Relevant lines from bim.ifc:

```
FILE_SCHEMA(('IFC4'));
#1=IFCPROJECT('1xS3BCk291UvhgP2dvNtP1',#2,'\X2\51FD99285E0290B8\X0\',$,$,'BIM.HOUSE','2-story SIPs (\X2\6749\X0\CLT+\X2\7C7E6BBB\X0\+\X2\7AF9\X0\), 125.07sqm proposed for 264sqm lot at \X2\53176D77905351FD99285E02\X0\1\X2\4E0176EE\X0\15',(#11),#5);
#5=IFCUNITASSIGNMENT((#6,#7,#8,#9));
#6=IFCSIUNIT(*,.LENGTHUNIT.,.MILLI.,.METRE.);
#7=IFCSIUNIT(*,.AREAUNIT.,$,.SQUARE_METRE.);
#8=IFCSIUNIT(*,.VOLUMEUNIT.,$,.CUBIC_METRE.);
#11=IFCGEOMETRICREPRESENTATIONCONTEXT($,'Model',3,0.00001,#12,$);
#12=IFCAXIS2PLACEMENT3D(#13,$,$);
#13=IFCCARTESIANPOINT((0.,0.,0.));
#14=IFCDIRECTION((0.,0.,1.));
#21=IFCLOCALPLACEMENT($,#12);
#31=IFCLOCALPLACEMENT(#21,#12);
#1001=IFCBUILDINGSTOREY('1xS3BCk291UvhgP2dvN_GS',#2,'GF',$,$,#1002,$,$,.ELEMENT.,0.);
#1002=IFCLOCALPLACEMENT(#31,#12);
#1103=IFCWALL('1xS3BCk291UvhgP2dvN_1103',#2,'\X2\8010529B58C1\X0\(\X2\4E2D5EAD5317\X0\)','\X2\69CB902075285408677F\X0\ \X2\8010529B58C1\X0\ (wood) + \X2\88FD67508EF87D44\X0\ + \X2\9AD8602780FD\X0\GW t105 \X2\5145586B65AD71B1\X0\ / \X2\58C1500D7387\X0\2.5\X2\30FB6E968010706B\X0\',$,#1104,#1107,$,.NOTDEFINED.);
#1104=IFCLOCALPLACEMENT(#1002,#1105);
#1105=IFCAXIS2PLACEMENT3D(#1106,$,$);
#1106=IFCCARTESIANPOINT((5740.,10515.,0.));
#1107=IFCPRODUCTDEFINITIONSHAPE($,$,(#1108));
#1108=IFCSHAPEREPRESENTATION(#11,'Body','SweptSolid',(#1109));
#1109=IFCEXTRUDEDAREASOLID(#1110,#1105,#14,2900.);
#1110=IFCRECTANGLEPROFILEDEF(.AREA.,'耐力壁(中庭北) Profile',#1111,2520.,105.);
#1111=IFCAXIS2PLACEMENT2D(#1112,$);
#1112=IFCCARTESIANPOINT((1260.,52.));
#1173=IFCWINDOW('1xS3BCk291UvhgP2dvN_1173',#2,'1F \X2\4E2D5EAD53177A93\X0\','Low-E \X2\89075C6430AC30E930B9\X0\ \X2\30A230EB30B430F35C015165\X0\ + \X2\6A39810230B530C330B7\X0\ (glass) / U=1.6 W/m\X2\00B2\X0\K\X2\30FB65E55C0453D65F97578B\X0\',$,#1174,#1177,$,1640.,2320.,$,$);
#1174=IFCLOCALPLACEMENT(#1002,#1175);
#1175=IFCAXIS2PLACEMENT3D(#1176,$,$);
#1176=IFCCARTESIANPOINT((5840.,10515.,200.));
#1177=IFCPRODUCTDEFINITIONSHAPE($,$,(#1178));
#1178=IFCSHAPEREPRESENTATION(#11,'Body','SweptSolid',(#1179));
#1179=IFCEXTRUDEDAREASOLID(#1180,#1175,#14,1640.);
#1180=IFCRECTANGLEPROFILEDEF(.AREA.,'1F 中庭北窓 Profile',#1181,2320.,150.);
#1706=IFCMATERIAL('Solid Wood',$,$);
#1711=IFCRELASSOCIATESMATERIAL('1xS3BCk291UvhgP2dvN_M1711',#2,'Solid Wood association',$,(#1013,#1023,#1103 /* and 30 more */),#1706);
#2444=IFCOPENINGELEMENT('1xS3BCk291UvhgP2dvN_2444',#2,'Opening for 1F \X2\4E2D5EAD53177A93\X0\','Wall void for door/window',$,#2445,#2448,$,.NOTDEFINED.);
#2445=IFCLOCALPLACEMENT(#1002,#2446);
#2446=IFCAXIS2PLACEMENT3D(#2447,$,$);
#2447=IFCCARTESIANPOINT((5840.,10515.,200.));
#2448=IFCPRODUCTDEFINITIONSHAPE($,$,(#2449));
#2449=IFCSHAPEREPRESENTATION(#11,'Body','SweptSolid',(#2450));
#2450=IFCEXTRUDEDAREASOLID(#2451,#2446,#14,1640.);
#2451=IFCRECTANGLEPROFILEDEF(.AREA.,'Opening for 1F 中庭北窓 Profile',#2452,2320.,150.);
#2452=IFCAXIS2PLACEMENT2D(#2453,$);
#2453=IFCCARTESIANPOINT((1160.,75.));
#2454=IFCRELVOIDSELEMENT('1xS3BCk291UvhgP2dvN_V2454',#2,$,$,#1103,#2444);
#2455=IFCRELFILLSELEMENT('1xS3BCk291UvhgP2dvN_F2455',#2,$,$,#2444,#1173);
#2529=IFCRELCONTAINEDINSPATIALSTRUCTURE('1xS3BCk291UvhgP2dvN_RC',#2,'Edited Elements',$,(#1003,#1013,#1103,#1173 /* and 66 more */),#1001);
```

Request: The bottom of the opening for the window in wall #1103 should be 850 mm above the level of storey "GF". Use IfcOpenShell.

```python
import numpy as np
import ifcopenshell
import ifcopenshell.api.geometry
import ifcopenshell.geom
import ifcopenshell.util.element
import ifcopenshell.util.placement
import ifcopenshell.util.shape
import ifcopenshell.util.unit

model = ifcopenshell.open("bim.ifc")
unit_scale = ifcopenshell.util.unit.calculate_unit_scale(model)

window = model.by_guid("1xS3BCk291UvhgP2dvN_1173")
opening = window.FillsVoids[0].RelatingOpeningElement
storey = ifcopenshell.util.element.get_container(window, ifc_class="IfcBuildingStorey")
level = ifcopenshell.util.placement.get_local_placement(storey.ObjectPlacement)[2, 3]

# The opening's origin need not be at the sill, so measure its lowest point.
shape = ifcopenshell.geom.create_shape(ifcopenshell.geom.settings(), opening)
bottom = ifcopenshell.util.shape.get_shape_bottom_elevation(shape, shape.geometry) / unit_scale
dz = level + 0.85 / unit_scale - bottom

shift = np.array([0.0, 0.0, dz])
# The window is not placed relative to its opening, so move both.
for product in (opening, window):
    matrix = ifcopenshell.util.placement.get_local_placement(product.ObjectPlacement)
    matrix[:3, 3] += shift
    ifcopenshell.api.geometry.edit_object_placement(model, product=product, matrix=matrix, is_si=False)

print(f"moved by {dz * unit_scale:+.3f} m")

model.write("bim_rev.ifc")
```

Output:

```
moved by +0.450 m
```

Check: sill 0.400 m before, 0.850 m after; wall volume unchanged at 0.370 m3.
